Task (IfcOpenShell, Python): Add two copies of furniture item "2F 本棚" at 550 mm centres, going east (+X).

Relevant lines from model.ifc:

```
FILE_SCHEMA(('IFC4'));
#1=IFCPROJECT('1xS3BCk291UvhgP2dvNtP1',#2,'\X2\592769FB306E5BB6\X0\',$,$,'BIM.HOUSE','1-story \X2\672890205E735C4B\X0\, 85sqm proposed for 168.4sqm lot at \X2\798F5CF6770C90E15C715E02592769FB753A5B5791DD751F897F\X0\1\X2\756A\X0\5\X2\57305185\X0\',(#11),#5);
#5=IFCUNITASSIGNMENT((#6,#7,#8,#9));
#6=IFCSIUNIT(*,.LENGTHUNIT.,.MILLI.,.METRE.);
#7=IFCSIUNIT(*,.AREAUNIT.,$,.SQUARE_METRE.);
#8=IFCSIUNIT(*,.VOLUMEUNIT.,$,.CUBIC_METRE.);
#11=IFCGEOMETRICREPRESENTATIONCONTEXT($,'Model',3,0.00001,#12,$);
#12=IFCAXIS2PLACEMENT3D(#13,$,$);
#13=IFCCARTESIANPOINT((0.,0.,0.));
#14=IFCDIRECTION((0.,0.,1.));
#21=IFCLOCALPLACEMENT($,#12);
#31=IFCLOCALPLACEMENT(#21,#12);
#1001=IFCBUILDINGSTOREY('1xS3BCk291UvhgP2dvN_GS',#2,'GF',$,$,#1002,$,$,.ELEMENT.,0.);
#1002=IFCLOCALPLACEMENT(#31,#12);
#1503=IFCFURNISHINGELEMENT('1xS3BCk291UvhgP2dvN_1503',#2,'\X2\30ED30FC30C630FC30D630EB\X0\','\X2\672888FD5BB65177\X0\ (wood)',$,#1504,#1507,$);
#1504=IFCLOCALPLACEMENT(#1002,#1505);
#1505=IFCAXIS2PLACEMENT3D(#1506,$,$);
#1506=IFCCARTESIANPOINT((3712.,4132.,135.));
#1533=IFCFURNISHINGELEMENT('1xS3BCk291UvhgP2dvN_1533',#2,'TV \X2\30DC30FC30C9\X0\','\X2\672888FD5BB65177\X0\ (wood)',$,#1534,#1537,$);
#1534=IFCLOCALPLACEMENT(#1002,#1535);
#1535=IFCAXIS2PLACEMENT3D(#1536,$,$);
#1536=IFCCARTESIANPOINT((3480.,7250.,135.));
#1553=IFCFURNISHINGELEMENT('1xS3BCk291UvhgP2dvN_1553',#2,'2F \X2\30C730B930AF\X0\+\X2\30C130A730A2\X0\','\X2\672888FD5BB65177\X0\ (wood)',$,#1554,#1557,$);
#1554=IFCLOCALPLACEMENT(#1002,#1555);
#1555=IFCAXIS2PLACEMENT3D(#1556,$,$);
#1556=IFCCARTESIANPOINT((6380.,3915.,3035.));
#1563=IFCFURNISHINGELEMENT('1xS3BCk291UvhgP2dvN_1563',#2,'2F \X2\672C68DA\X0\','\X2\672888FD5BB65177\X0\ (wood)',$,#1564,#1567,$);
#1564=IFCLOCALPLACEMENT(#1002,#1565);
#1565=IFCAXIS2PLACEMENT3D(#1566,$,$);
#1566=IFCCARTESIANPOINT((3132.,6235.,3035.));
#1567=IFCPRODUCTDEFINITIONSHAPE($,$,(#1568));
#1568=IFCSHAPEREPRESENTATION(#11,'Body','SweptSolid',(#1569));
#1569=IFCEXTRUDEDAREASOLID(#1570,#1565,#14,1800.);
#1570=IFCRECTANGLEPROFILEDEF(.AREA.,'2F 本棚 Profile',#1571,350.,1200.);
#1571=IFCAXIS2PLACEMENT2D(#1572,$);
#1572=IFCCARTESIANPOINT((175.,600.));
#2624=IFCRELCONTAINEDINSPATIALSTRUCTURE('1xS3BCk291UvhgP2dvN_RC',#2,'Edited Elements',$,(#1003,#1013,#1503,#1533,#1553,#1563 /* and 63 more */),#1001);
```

```python
import numpy as np
import ifcopenshell
import ifcopenshell.api.geometry
import ifcopenshell.api.root
import ifcopenshell.util.element
import ifcopenshell.util.placement

model = ifcopenshell.open("model.ifc")


def reuse_history(source, copy):
    """copy_class also copies each property set's owner history, people and application; keep the originals."""
    for rel in copy.IsDefinedBy:
        if rel.is_a("IfcRelDefinesByProperties") and (history := rel.RelatingPropertyDefinition.OwnerHistory):
            rel.RelatingPropertyDefinition.OwnerHistory = source.OwnerHistory
            ifcopenshell.util.element.remove_deep2(model, history)


source = model.by_id(1563)
base = ifcopenshell.util.placement.get_local_placement(source.ObjectPlacement)
step = np.array([1.0, 0.0, 0.0]) * 550.0

for i in range(1, 3):
    copy = ifcopenshell.api.root.copy_class(model, product=source)
    copy.Representation = ifcopenshell.util.element.copy_deep(
        model, source.Representation, exclude=["IfcGeometricRepresentationContext", "IfcRepresentationMap"]
    )
    reuse_history(source, copy)
    matrix = base.copy()
    matrix[:3, 3] += i * step
    print("added at", matrix[:3, 3].round(3) + 0.0)
    ifcopenshell.api.geometry.edit_object_placement(model, product=copy, matrix=matrix, is_si=False)

model.write("model_updated.ifc")
```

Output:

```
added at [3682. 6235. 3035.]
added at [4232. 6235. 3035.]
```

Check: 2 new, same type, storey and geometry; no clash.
